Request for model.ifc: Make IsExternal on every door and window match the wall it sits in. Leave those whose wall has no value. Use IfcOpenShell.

First a look at what the model holds.

```python
import ifcopenshell
import ifcopenshell.util.element

model = ifcopenshell.open("model.ifc")
print(model.schema)
seen = {}
for e in model.by_type("IfcDoor") + model.by_type("IfcWindow"):
    if not e.FillsVoids:
        continue
    host = e.FillsVoids[0].RelatingOpeningElement.VoidsElements[0].RelatingBuildingElement
    own = ifcopenshell.util.element.get_pset(e, f"Pset_{e.is_a()[3:].removesuffix('StandardCase')}Common", "IsExternal")
    wall = ifcopenshell.util.element.get_pset(host, "Pset_WallCommon", "IsExternal")
    seen[e.is_a(), own, wall] = seen.get((e.is_a(), own, wall), 0) + 1
for (cls, own, wall), count in sorted(seen.items(), key=str):
    print(count, cls, "IsExternal:", own, "| host wall:", wall)
```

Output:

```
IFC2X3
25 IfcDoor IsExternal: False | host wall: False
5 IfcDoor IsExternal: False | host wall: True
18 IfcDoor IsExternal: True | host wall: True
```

```python
import ifcopenshell
import ifcopenshell.api.pset
import ifcopenshell.util.element

model = ifcopenshell.open("model.ifc")

count = 0
for ifc_class, pset_name in (("IfcDoor", "Pset_DoorCommon"), ("IfcWindow", "Pset_WindowCommon")):
    for e in model.by_type(ifc_class):
        if not e.FillsVoids:
            continue
        host = e.FillsVoids[0].RelatingOpeningElement.VoidsElements[0].RelatingBuildingElement
        external = ifcopenshell.util.element.get_pset(host, "Pset_WallCommon", "IsExternal")
        if external is None or ifcopenshell.util.element.get_pset(e, pset_name, "IsExternal") == external:
            continue
        pset = ifcopenshell.api.pset.add_pset(model, product=e, name=pset_name)
        ifcopenshell.api.pset.edit_pset(model, pset=pset, properties={"IsExternal": external})
        count += 1

print(count, "updated")

model.write("model_updated.ifc")
```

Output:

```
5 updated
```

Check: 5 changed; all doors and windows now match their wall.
